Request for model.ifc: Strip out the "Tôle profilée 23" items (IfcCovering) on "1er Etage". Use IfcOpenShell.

First a look at what the model holds.

```python
import ifcopenshell
import ifcopenshell.util.element

model = ifcopenshell.open("model.ifc")
print(model.schema)
storey = next(s for s in model.by_type("IfcBuildingStorey") if s.Name == "1er Etage")
coverings = [e for e in ifcopenshell.util.element.get_decomposition(storey) if e.is_a("IfcCovering")]
seen = {}
for e in coverings:
    element_type = ifcopenshell.util.element.get_type(e)
    name = element_type.Name if element_type not in (None, e) else None
    seen[name] = seen.get(name, 0) + 1
for name, count in sorted(seen.items(), key=str):
    print(count, "x", name)
```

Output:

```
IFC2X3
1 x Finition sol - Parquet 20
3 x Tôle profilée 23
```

```python
import ifcopenshell
import ifcopenshell.api.root
import ifcopenshell.util.element

model = ifcopenshell.open("model.ifc")

storey = next(s for s in model.by_type("IfcBuildingStorey") if s.Name == "1er Etage")
coverings = [e for e in ifcopenshell.util.element.get_decomposition(storey) if e.is_a("IfcCovering")]
targets = [e for e in coverings if (t := ifcopenshell.util.element.get_type(e)) not in (None, e) and t.Name == "Tôle profilée 23"]

for e in targets:
    ifcopenshell.api.root.remove_product(model, product=e)
print(len(targets), "removed")

model.write("model_updated.ifc")
```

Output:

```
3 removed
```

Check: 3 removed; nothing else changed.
